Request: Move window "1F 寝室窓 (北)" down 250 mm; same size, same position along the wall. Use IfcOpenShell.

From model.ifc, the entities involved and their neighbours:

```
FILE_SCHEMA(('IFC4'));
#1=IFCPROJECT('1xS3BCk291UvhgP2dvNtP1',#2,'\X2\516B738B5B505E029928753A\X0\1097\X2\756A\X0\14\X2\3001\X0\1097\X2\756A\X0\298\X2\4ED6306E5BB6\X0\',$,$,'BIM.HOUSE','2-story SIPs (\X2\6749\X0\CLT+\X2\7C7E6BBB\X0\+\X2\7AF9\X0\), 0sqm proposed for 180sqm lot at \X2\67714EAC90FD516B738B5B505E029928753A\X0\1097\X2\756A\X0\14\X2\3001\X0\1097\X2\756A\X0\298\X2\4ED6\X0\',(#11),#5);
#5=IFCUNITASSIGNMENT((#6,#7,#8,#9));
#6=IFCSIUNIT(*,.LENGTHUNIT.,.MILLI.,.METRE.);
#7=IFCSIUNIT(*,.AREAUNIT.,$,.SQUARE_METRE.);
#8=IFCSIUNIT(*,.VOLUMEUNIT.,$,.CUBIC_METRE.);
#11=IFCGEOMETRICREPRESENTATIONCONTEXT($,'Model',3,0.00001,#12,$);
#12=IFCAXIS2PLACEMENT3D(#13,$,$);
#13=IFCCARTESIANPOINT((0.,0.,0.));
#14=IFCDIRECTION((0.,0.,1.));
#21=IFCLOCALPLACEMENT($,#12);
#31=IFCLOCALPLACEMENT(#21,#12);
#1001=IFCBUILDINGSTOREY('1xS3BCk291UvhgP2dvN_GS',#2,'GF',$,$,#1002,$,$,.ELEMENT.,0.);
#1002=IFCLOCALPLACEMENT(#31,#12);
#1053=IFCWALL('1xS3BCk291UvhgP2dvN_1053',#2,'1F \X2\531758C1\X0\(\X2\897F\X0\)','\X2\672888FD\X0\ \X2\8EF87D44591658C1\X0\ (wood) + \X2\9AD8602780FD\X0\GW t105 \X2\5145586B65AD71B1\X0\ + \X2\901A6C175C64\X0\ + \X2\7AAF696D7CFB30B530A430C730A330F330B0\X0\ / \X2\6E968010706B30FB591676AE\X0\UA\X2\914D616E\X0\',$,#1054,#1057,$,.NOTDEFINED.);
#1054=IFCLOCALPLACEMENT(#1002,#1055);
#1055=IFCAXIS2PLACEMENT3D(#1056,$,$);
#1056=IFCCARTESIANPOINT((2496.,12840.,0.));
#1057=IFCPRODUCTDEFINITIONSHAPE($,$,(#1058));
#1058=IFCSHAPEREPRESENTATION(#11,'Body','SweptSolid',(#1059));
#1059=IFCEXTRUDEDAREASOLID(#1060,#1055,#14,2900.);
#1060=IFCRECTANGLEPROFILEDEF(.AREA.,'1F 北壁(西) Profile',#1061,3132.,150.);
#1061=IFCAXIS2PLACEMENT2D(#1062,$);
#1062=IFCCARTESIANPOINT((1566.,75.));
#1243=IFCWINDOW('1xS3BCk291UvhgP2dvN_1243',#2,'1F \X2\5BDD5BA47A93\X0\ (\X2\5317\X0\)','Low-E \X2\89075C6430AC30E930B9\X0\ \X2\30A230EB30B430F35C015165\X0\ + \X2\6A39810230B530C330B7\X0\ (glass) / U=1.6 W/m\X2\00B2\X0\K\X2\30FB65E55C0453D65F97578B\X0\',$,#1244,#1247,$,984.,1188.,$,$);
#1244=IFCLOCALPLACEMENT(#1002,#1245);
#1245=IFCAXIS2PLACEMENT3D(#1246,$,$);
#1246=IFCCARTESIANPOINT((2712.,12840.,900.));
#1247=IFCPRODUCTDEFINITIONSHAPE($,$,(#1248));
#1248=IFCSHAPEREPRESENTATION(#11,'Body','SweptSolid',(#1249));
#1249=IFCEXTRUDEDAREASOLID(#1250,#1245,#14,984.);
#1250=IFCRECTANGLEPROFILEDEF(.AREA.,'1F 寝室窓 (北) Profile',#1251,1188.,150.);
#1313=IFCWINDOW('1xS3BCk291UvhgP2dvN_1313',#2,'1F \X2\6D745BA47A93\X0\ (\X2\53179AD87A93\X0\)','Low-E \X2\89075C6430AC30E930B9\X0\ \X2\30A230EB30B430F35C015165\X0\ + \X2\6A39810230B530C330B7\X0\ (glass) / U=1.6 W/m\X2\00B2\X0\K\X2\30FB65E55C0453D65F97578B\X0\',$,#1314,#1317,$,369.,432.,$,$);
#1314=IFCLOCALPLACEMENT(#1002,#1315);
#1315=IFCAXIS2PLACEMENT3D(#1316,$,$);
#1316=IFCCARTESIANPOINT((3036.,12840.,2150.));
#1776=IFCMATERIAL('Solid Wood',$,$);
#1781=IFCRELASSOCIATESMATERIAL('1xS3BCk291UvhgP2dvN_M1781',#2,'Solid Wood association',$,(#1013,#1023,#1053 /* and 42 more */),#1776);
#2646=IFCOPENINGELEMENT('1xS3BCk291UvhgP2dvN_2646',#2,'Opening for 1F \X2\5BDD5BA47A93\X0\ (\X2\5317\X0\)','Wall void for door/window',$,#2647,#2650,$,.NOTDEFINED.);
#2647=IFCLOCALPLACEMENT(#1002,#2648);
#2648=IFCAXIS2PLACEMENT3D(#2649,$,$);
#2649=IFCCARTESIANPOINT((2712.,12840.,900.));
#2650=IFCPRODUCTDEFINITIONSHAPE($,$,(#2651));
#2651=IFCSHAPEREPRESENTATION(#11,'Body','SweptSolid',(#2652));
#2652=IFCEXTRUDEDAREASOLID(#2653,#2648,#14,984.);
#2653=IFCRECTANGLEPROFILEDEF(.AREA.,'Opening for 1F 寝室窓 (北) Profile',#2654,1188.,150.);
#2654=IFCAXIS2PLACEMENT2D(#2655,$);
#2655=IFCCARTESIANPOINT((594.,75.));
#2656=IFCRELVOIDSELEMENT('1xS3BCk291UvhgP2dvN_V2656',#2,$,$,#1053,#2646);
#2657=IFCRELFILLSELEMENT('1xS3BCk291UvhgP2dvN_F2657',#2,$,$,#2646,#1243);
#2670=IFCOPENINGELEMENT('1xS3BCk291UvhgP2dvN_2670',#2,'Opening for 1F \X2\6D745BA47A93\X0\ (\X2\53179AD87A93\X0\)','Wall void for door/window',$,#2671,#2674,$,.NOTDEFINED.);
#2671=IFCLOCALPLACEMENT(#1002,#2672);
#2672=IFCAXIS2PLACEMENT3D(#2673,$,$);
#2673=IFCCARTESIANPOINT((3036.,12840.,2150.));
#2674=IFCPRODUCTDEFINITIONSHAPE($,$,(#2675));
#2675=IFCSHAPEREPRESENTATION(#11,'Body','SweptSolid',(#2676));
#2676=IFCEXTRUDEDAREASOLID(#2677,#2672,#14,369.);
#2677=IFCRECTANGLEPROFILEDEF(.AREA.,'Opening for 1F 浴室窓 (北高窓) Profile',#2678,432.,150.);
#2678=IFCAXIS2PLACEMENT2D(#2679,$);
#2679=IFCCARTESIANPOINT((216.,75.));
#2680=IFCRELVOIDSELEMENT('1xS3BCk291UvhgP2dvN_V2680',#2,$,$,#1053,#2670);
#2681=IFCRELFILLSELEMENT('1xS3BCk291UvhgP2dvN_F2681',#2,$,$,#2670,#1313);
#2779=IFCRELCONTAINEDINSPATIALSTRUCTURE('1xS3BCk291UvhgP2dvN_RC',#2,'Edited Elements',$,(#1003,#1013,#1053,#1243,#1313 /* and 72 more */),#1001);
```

```python
import numpy as np
import ifcopenshell
import ifcopenshell.api.geometry
import ifcopenshell.util.placement
import ifcopenshell.util.unit

model = ifcopenshell.open("model.ifc")
unit_scale = ifcopenshell.util.unit.calculate_unit_scale(model)

window = model.by_guid("1xS3BCk291UvhgP2dvN_1243")
opening = window.FillsVoids[0].RelatingOpeningElement
dz = -0.25 / unit_scale

shift = np.array([0.0, 0.0, dz])
# The window is not placed relative to its opening, so move both.
for product in (opening, window):
    matrix = ifcopenshell.util.placement.get_local_placement(product.ObjectPlacement)
    matrix[:3, 3] += shift
    ifcopenshell.api.geometry.edit_object_placement(model, product=product, matrix=matrix, is_si=False)

print(f"moved by {dz * unit_scale:+.3f} m")

model.write("model-out.ifc")
```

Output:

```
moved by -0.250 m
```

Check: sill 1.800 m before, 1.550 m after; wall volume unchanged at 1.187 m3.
